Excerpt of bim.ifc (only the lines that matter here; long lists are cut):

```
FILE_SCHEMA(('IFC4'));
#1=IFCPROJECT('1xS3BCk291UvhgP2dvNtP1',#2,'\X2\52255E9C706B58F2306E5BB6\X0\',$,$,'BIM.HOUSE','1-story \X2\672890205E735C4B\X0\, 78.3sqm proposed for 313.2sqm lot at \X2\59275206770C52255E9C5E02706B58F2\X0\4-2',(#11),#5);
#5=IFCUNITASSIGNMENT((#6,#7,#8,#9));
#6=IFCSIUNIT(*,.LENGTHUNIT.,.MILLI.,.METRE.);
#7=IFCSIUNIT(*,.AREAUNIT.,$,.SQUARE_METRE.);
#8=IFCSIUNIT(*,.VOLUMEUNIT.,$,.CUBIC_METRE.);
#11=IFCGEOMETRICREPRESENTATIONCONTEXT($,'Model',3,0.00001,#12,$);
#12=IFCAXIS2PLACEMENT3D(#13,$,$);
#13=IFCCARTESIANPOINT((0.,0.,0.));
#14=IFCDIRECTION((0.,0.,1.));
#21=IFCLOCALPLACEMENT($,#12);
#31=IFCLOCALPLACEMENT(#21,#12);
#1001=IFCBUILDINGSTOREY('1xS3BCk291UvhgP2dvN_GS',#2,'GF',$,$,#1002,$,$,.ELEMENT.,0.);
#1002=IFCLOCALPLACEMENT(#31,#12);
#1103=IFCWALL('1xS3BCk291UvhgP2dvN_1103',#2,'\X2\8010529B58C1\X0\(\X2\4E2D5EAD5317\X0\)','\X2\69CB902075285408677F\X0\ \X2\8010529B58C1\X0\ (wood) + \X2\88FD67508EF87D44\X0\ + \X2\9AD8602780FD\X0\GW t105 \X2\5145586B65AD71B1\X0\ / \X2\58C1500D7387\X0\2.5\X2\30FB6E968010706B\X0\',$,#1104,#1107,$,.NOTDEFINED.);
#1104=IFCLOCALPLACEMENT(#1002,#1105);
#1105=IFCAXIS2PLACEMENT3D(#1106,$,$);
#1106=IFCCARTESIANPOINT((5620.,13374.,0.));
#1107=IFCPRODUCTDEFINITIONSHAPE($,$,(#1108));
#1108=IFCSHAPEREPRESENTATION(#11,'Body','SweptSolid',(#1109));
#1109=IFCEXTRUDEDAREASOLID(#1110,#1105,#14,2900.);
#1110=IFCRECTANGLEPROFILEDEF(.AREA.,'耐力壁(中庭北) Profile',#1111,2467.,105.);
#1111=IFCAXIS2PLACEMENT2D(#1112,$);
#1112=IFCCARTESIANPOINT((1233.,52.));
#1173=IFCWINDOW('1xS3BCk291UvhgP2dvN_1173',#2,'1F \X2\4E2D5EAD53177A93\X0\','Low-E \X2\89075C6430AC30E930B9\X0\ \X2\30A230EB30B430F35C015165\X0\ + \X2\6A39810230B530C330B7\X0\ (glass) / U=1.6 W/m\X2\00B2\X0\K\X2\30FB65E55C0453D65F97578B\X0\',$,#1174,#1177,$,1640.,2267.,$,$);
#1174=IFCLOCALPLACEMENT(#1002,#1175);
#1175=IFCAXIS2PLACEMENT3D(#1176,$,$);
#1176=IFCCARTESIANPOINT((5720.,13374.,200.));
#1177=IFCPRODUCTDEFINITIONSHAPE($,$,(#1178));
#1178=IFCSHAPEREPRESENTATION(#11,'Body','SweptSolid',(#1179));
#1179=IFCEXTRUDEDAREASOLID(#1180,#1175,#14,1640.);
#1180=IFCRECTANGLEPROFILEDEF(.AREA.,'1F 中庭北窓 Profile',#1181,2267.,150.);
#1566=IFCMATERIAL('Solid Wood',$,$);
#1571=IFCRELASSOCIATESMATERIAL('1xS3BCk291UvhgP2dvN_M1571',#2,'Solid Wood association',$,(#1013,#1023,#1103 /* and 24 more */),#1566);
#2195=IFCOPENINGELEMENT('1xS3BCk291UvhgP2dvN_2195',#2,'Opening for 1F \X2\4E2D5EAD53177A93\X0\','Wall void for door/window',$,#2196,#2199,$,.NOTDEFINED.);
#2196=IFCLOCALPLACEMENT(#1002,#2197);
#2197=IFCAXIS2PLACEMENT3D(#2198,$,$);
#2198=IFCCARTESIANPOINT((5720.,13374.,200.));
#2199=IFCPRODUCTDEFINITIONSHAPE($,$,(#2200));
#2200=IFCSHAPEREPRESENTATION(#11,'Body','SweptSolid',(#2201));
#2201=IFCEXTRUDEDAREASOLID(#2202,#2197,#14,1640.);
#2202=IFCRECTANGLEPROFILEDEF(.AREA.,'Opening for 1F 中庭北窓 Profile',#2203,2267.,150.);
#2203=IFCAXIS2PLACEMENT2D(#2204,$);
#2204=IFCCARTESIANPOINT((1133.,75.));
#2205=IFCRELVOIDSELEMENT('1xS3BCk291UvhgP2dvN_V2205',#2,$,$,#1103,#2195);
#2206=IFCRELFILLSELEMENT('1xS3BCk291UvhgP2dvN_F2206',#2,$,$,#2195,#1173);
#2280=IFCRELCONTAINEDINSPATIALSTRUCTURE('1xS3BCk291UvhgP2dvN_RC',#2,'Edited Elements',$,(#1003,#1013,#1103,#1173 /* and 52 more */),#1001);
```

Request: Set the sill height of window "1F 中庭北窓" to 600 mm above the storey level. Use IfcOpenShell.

```python
import numpy as np
import ifcopenshell
import ifcopenshell.api.geometry
import ifcopenshell.geom
import ifcopenshell.util.element
import ifcopenshell.util.placement
import ifcopenshell.util.shape
import ifcopenshell.util.unit

model = ifcopenshell.open("bim.ifc")
unit_scale = ifcopenshell.util.unit.calculate_unit_scale(model)

window = model.by_guid("1xS3BCk291UvhgP2dvN_1173")
opening = window.FillsVoids[0].RelatingOpeningElement
storey = ifcopenshell.util.element.get_container(window, ifc_class="IfcBuildingStorey")
level = ifcopenshell.util.placement.get_local_placement(storey.ObjectPlacement)[2, 3]

# The opening's origin need not be at the sill, so measure its lowest point.
shape = ifcopenshell.geom.create_shape(ifcopenshell.geom.settings(), opening)
bottom = ifcopenshell.util.shape.get_shape_bottom_elevation(shape, shape.geometry) / unit_scale
dz = level + 600.0 - bottom

shift = np.array([0.0, 0.0, dz])
# The window is not placed relative to its opening, so move both.
for product in (opening, window):
    matrix = ifcopenshell.util.placement.get_local_placement(product.ObjectPlacement)
    matrix[:3, 3] += shift
    ifcopenshell.api.geometry.edit_object_placement(model, product=product, matrix=matrix, is_si=False)

print(f"moved by {dz * unit_scale:+.3f} m")

model.write("bim_updated.ifc")
```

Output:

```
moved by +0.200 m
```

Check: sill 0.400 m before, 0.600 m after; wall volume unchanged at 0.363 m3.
